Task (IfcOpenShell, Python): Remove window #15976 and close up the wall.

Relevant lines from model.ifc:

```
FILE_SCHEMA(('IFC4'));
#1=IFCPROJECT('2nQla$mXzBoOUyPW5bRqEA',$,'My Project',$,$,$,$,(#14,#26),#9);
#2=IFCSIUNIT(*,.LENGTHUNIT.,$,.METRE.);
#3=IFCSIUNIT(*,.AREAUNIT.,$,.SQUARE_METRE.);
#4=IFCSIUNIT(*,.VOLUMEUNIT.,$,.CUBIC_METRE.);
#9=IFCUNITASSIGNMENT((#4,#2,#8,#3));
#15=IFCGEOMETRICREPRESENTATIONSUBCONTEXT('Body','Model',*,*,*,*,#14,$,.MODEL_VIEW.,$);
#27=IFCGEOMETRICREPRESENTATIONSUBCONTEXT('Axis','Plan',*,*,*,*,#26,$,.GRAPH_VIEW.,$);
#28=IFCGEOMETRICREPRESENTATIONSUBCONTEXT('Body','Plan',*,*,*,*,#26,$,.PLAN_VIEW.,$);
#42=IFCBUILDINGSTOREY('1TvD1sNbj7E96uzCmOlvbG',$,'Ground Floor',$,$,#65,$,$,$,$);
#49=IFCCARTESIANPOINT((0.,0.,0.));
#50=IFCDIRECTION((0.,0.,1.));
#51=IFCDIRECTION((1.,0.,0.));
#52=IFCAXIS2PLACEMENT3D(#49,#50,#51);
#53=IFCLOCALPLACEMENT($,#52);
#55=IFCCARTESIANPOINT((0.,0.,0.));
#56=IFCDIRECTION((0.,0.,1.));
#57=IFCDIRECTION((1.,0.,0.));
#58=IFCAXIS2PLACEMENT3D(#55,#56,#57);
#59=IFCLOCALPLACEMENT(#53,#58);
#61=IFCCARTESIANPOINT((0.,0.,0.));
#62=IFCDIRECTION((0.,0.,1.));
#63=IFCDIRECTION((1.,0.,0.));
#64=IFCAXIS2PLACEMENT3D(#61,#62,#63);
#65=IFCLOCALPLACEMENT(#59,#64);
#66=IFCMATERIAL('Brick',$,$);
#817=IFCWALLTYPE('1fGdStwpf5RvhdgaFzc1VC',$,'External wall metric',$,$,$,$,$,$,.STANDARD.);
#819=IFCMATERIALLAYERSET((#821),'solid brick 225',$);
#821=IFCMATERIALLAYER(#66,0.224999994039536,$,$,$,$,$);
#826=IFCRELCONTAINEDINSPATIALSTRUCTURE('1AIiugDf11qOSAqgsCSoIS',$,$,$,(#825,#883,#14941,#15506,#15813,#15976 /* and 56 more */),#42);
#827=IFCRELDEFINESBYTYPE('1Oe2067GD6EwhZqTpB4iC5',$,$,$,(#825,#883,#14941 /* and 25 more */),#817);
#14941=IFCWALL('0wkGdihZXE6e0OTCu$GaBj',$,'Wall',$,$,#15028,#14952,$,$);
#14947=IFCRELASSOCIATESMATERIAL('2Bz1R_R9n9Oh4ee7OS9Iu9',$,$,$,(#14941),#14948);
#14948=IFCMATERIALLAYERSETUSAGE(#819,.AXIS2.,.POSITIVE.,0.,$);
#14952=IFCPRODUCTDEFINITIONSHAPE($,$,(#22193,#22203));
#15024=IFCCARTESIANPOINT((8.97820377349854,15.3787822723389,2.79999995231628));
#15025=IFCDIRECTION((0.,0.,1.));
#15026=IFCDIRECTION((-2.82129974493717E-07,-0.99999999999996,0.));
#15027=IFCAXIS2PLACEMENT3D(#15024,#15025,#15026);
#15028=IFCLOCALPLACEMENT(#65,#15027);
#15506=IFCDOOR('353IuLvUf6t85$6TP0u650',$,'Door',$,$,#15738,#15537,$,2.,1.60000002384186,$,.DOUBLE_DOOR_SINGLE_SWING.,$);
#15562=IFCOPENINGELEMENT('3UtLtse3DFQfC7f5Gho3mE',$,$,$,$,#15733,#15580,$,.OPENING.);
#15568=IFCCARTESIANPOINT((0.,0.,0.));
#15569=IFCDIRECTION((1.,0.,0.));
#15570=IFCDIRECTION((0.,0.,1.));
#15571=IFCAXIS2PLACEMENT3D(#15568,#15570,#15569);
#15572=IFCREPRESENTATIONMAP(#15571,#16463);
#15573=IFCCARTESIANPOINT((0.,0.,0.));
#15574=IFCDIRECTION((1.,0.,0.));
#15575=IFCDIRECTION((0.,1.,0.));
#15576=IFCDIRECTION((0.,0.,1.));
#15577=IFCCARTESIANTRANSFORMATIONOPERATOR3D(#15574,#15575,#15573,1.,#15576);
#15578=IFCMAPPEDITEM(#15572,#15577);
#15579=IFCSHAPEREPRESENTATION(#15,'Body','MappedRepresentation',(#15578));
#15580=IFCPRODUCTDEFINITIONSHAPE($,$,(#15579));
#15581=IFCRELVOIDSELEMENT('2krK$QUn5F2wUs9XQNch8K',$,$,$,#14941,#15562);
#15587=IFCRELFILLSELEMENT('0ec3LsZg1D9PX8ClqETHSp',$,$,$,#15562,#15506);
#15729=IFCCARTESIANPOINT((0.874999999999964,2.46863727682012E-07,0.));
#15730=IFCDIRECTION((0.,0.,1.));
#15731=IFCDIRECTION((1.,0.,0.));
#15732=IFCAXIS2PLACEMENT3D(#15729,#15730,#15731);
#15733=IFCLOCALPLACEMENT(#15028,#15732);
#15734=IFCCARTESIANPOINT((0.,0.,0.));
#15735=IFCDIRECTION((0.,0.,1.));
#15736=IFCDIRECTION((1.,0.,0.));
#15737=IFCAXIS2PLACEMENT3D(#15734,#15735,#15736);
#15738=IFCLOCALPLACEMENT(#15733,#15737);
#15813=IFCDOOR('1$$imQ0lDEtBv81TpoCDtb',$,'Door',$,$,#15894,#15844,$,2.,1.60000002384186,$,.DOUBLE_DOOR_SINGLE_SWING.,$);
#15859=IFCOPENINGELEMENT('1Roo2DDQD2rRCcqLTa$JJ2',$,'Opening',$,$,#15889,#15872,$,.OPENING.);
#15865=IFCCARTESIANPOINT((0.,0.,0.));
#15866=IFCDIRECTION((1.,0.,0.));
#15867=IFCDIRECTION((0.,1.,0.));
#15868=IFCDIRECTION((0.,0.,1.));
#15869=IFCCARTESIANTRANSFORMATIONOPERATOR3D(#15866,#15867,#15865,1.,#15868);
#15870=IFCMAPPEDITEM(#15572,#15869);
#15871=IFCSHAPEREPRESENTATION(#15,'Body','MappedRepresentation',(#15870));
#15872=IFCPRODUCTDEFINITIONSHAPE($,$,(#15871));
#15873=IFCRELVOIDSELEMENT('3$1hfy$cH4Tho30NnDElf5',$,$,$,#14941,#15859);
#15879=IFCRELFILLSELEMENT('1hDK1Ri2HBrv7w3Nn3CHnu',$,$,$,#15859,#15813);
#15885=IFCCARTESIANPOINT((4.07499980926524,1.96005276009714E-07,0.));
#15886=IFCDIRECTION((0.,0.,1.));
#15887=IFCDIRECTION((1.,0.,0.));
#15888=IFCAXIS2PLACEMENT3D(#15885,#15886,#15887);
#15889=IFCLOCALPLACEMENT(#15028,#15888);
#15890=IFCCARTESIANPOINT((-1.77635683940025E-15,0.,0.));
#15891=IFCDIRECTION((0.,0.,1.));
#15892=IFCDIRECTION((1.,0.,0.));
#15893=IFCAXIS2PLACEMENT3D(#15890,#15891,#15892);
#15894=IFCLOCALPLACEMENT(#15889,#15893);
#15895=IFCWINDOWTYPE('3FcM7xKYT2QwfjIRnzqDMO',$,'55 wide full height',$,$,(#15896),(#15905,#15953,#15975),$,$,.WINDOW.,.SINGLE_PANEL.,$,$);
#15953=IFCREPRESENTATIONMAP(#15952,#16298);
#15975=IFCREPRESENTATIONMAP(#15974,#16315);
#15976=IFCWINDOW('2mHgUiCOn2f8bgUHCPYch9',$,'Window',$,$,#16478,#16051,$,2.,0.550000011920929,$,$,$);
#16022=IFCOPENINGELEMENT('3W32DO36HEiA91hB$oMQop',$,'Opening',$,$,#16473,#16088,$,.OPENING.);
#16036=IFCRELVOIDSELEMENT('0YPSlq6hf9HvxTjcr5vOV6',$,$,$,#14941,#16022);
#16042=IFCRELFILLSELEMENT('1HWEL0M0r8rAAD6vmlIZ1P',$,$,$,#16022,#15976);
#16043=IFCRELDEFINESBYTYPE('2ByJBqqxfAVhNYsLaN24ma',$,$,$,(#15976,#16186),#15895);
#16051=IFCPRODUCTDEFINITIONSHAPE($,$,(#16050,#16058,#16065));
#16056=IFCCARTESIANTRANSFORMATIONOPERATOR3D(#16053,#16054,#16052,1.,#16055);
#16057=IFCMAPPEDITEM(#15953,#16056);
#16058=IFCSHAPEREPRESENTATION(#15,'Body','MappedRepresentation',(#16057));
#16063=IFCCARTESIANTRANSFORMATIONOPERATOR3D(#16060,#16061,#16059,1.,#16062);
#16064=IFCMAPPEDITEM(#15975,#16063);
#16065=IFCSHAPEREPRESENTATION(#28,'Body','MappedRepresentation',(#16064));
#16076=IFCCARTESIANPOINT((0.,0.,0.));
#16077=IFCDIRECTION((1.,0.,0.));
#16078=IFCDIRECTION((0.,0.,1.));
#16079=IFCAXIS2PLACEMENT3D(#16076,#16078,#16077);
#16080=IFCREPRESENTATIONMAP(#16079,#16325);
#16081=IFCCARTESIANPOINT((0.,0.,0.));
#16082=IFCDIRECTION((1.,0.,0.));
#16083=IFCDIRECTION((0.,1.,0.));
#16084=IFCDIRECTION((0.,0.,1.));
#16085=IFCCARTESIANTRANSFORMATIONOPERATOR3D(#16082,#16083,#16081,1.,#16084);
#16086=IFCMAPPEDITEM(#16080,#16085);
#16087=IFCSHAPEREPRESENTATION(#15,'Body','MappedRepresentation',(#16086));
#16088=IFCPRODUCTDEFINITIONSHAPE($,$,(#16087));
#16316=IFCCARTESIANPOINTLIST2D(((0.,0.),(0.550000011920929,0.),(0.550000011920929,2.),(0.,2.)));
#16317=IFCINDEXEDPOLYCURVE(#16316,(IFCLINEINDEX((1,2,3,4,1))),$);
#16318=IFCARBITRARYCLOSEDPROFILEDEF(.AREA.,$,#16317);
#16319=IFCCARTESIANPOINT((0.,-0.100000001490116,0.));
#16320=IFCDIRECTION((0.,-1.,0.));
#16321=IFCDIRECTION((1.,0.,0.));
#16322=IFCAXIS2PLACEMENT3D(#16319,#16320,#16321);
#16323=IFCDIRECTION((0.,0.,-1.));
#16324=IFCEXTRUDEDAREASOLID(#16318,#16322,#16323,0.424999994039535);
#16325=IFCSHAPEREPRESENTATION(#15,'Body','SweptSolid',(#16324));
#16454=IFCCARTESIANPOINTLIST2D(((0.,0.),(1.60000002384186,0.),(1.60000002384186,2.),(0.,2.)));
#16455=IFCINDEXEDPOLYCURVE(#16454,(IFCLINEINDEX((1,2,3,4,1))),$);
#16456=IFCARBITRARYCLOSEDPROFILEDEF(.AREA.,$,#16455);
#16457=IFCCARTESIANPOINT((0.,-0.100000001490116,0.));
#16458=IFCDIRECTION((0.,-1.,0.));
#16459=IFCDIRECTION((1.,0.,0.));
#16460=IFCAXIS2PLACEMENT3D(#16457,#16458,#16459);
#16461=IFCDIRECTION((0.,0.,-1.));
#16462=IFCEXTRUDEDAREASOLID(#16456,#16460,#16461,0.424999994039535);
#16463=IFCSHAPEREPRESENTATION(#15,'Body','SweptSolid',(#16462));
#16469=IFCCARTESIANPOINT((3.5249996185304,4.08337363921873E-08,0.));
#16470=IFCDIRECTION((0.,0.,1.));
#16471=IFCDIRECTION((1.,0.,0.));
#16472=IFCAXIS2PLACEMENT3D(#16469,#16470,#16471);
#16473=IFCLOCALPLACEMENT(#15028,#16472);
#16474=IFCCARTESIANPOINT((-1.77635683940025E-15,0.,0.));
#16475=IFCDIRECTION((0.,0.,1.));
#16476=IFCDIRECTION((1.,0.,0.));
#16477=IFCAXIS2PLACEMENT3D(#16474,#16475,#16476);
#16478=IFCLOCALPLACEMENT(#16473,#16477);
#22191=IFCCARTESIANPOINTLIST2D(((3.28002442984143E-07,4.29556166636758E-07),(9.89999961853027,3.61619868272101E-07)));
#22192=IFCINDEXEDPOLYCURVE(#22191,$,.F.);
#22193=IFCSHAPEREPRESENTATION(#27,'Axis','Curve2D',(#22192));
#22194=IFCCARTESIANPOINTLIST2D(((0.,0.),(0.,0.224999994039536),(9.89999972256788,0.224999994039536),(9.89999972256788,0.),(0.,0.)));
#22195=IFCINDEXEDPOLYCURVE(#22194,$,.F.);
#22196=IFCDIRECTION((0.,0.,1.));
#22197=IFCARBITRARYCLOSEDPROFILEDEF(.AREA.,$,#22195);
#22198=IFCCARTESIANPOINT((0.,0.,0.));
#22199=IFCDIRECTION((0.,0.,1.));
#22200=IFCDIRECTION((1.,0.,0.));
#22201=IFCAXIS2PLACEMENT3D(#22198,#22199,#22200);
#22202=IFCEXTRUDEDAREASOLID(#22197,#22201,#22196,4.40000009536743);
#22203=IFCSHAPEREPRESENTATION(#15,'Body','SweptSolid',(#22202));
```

```python
import ifcopenshell
import ifcopenshell.api.feature
import ifcopenshell.api.root
import ifcopenshell.geom
import ifcopenshell.util.shape

model = ifcopenshell.open("model.ifc")
settings = ifcopenshell.geom.settings()


def volume(element):
    """Net volume in cubic metres, openings subtracted."""
    shape = ifcopenshell.geom.create_shape(settings, element)
    return ifcopenshell.util.shape.get_volume(shape.geometry)


window = model.by_guid("2mHgUiCOn2f8bgUHCPYch9")
opening = window.FillsVoids[0].RelatingOpeningElement
wall = opening.VoidsElements[0].RelatingBuildingElement
before = volume(wall)

ifcopenshell.api.root.remove_product(model, product=window)
ifcopenshell.api.feature.remove_feature(model, feature=opening)

after = volume(wall)

print(f"wall volume {before:.3f} -> {after:.3f} m3")

model.write("model_rev.ifc")
```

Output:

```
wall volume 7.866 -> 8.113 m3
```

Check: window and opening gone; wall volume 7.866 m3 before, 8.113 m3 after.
